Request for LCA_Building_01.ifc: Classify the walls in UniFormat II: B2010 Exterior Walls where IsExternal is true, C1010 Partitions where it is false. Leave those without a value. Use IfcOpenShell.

First a look at what the model holds.

```python
import ifcopenshell
import ifcopenshell.util.element

model = ifcopenshell.open("LCA_Building_01.ifc")
print(model.schema)
print("classifications:", [c.Name for c in model.by_type("IfcClassification")])
values = [ifcopenshell.util.element.get_pset(e, "Pset_WallCommon", "IsExternal") for e in model.by_type("IfcWall")]
for value in (True, False, None):
    print("IsExternal", value, values.count(value))
```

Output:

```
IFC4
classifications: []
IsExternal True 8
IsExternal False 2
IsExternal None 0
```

```python
import ifcopenshell
import ifcopenshell.api.classification
import ifcopenshell.util.element

model = ifcopenshell.open("LCA_Building_01.ifc")

system = ifcopenshell.api.classification.add_classification(model, classification="UniFormat II")

walls = model.by_type("IfcWall")
external = {e: ifcopenshell.util.element.get_pset(e, "Pset_WallCommon", "IsExternal") for e in walls}
for flag, code, name in ((True, "B2010", "Exterior Walls"), (False, "C1010", "Partitions")):
    products = [e for e in walls if external[e] is flag]
    ifcopenshell.api.classification.add_reference(
        model, products=products, classification=system, identification=code, name=name
    )
    print(code, len(products))

model.write("LCA_Building_01_rev.ifc")
```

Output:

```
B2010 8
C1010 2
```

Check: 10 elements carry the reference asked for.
